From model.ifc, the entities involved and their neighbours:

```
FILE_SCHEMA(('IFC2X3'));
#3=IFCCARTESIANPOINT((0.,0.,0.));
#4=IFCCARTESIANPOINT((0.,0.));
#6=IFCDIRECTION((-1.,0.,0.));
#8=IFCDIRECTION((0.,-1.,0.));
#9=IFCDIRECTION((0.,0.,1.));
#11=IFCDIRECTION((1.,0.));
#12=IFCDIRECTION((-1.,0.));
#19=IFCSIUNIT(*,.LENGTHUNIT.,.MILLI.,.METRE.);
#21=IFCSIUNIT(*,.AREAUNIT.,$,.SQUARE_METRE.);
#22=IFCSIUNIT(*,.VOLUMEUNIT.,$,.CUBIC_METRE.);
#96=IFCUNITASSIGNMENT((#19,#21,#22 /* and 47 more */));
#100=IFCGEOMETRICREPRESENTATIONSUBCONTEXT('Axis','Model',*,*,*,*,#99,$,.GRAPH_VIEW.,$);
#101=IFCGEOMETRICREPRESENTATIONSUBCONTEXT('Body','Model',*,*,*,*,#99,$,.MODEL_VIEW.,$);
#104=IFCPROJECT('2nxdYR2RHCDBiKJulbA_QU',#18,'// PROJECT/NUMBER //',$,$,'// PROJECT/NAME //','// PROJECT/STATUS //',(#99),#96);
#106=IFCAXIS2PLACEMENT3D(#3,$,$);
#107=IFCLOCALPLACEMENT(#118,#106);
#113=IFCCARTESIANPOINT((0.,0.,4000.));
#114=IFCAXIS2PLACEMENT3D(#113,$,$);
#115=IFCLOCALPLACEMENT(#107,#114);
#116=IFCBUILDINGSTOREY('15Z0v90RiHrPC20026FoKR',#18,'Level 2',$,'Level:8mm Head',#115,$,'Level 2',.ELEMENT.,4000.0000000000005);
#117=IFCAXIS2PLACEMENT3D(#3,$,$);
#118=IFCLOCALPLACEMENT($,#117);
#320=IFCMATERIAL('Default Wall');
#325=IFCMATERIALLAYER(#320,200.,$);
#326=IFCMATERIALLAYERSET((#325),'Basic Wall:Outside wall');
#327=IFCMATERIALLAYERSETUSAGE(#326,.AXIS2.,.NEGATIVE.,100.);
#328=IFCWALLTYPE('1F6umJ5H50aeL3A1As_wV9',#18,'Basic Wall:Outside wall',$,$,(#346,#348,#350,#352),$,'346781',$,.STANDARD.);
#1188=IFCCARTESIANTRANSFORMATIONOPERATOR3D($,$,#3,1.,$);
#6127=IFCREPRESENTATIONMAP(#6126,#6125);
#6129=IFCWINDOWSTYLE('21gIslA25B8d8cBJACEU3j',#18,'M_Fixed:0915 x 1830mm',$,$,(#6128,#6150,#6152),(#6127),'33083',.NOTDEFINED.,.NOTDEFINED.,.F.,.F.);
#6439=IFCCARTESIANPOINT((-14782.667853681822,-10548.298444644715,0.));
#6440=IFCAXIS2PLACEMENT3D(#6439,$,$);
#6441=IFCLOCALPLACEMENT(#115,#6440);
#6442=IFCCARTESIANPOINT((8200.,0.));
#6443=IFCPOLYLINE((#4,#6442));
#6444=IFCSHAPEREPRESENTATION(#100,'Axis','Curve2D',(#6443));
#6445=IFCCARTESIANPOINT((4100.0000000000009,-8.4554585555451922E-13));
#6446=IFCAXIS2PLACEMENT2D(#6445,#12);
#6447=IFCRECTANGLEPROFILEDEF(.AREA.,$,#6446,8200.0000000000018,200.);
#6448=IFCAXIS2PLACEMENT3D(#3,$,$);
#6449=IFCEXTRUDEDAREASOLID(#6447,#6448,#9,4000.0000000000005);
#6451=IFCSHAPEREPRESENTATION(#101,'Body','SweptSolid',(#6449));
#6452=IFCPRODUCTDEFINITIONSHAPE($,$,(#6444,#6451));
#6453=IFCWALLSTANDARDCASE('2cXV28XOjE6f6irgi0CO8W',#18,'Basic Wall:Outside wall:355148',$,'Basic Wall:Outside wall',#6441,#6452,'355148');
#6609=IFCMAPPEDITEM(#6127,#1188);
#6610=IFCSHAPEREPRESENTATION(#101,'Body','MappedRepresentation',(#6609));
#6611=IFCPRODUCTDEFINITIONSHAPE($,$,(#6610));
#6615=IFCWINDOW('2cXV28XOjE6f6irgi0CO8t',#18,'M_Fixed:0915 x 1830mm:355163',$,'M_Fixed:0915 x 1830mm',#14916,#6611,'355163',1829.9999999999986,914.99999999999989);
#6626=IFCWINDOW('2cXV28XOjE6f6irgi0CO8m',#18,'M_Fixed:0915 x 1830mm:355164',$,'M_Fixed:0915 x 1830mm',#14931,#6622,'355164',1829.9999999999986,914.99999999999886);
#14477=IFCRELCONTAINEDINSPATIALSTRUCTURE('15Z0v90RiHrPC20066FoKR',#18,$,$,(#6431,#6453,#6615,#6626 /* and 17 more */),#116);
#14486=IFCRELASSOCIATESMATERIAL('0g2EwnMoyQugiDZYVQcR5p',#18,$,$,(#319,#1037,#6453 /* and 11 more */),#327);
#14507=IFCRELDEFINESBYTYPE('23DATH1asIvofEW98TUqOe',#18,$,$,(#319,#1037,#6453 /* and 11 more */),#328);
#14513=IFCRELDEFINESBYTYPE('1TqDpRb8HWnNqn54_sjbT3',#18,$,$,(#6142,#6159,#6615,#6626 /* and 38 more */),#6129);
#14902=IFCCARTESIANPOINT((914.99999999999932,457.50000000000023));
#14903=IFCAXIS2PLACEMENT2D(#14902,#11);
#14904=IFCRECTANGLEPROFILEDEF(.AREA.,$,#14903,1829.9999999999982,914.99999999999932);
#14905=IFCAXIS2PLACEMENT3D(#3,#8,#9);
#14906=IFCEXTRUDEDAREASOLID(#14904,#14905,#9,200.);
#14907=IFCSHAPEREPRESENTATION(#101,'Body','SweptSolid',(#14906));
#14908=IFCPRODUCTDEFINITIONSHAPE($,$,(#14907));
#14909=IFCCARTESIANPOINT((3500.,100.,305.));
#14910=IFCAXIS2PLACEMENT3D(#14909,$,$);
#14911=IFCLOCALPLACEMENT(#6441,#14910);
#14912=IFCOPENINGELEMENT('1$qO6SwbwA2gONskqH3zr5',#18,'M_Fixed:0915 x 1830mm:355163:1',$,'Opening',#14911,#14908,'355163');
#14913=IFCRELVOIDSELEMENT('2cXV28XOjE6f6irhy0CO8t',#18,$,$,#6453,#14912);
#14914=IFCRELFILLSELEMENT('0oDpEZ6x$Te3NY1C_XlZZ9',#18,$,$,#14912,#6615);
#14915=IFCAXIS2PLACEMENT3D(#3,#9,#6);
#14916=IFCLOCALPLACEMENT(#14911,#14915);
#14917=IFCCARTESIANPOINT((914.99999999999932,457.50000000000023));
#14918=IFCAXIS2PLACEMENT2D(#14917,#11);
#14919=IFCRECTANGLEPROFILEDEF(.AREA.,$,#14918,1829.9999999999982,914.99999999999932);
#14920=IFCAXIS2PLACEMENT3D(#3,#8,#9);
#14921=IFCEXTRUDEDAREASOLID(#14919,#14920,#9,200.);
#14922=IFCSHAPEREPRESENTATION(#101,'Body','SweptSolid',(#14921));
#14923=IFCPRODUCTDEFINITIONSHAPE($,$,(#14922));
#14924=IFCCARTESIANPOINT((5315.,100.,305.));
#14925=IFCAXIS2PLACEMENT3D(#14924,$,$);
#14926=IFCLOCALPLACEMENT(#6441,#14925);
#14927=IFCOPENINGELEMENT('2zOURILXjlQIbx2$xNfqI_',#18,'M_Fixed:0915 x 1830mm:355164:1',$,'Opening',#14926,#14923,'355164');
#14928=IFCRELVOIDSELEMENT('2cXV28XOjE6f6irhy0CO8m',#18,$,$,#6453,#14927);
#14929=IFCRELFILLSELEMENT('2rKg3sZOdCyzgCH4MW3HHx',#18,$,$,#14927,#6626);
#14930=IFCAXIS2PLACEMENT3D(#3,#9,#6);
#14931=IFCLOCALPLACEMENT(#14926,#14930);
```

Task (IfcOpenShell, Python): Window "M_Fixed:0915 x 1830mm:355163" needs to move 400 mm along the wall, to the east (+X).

```python
import ifcopenshell
import ifcopenshell.api.geometry
import ifcopenshell.util.placement
import ifcopenshell.util.unit

model = ifcopenshell.open("model.ifc")
unit_scale = ifcopenshell.util.unit.calculate_unit_scale(model)

window = model.by_guid("2cXV28XOjE6f6irgi0CO8t")
opening = window.FillsVoids[0].RelatingOpeningElement
wall = opening.VoidsElements[0].RelatingBuildingElement

wall_matrix = ifcopenshell.util.placement.get_local_placement(wall.ObjectPlacement)
shift = wall_matrix[:3, 0] * 0.4 / unit_scale
before = ifcopenshell.util.placement.get_local_placement(window.ObjectPlacement)[:3, 3].copy()

# The window is placed relative to its opening, so it follows when the opening moves.
matrix = ifcopenshell.util.placement.get_local_placement(opening.ObjectPlacement)
matrix[:3, 3] += shift
ifcopenshell.api.geometry.edit_object_placement(
    model, product=opening, matrix=matrix, is_si=False, should_transform_children=True
)

after = ifcopenshell.util.placement.get_local_placement(window.ObjectPlacement)[:3, 3]
print("window moved by", (after - before).round(3) + 0.0)

model.write("model-out.ifc")
```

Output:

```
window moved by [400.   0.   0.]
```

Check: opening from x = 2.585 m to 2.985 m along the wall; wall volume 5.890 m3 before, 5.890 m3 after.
